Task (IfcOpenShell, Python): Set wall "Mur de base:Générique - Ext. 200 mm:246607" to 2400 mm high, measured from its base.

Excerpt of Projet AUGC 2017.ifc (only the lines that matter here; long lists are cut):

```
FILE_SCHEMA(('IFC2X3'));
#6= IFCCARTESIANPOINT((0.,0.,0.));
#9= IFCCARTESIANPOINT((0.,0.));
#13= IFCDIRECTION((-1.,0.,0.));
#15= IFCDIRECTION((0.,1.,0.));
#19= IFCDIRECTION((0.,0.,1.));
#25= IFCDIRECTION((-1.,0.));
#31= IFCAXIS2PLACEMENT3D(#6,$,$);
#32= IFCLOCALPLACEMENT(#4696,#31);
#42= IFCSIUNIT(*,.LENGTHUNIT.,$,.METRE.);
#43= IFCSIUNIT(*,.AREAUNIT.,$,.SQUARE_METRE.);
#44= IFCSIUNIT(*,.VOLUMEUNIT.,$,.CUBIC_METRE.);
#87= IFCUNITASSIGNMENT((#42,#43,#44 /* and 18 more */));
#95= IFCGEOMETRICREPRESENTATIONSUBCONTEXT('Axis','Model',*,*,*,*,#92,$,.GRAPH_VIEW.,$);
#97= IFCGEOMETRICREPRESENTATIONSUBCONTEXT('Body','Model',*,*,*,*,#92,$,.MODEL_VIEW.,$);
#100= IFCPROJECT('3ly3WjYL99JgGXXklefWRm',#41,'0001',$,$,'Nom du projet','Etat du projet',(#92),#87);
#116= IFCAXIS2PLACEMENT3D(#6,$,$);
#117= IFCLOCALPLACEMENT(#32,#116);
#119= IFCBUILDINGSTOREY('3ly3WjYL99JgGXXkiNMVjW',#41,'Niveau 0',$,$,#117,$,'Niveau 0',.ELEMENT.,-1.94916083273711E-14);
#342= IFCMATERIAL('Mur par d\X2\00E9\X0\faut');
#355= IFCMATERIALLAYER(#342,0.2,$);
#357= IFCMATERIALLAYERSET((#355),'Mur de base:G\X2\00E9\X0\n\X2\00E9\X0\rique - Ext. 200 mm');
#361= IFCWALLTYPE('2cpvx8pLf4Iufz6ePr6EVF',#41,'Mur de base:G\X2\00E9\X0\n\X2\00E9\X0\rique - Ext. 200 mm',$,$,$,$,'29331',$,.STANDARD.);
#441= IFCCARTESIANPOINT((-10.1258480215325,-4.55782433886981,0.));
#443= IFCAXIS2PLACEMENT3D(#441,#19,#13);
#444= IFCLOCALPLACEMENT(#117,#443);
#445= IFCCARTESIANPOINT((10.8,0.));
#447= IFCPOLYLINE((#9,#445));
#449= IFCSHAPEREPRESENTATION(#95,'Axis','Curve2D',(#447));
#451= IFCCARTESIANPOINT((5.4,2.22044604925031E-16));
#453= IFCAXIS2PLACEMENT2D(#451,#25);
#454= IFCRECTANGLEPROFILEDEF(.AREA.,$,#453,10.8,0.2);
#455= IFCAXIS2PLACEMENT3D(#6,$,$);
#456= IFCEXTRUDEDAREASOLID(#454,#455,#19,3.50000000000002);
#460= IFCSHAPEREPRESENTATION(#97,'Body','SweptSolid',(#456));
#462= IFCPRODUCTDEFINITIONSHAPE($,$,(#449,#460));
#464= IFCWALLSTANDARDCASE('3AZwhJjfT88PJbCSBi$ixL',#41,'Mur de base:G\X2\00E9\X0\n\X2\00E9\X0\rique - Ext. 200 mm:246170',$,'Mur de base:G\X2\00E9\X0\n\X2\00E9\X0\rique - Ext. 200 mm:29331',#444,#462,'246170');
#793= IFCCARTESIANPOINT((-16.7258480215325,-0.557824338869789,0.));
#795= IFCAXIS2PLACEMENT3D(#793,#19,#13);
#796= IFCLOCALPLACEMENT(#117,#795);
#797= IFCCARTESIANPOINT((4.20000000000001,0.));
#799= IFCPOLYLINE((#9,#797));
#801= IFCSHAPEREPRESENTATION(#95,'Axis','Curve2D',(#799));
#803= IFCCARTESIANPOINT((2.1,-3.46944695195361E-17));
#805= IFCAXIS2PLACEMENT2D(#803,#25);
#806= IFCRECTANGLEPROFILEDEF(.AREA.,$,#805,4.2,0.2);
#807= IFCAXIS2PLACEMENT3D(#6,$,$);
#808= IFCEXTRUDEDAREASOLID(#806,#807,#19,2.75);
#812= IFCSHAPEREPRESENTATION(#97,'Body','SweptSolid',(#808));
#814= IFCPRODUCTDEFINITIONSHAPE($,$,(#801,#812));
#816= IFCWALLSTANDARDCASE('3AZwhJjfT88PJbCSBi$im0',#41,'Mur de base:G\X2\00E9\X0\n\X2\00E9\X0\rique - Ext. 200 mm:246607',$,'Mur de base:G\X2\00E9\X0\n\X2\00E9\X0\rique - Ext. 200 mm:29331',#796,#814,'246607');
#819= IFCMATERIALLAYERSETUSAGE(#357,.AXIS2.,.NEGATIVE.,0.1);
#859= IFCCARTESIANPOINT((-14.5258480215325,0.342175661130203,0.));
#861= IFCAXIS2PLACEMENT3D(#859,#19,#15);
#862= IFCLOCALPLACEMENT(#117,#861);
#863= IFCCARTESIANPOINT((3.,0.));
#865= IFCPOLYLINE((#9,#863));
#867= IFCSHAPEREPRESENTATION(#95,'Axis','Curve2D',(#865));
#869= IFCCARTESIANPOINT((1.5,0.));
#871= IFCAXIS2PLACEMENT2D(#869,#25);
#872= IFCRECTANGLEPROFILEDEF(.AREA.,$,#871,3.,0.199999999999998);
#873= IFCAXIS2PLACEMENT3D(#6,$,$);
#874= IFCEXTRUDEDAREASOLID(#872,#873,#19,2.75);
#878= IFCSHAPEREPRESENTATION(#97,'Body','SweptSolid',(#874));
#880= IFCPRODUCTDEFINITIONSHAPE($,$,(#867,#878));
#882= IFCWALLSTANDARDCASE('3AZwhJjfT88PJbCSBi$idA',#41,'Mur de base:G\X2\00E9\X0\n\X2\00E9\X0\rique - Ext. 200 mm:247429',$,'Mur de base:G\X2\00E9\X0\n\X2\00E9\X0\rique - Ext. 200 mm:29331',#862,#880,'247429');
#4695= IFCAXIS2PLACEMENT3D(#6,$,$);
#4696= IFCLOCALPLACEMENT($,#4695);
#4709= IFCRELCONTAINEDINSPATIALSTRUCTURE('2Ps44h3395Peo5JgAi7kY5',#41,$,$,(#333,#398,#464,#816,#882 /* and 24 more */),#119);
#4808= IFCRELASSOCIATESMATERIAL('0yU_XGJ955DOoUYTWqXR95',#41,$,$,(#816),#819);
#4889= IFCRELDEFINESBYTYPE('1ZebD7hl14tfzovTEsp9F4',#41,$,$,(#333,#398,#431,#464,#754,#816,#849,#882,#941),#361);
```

```python
import ifcopenshell
import ifcopenshell.geom
import ifcopenshell.util.representation
import ifcopenshell.util.shape
import ifcopenshell.util.unit

model = ifcopenshell.open("Projet AUGC 2017.ifc")
unit_scale = ifcopenshell.util.unit.calculate_unit_scale(model)
settings = ifcopenshell.geom.settings()


def volume(element):
    """Net volume in cubic metres, openings subtracted."""
    shape = ifcopenshell.geom.create_shape(settings, element)
    return ifcopenshell.util.shape.get_volume(shape.geometry)


wall = model.by_guid("3AZwhJjfT88PJbCSBi$im0")
before = volume(wall)

body = ifcopenshell.util.representation.get_representation(wall, "Model", "Body")
solid = body.Items[0]
old_height = solid.Depth
solid.Depth = 2.4 / unit_scale
after = volume(wall)

print(f"height {old_height:g} -> {solid.Depth:g}, volume {before:.3f} -> {after:.3f} m3")

model.write("Projet AUGC 2017_v2.ifc")
```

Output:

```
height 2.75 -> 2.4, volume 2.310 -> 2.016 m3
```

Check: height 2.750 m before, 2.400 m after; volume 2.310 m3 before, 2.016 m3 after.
